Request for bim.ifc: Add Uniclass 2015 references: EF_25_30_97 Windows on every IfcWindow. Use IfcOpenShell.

First a look at what the model holds.

```python
import ifcopenshell

model = ifcopenshell.open("bim.ifc")
print(model.schema)
print("classifications:", [c.Name for c in model.by_type("IfcClassification")])
for ifc_class in ("IfcDoor", "IfcRoof", "IfcStair", "IfcWall", "IfcWindow"):
    print(ifc_class, len(model.by_type(ifc_class)))
```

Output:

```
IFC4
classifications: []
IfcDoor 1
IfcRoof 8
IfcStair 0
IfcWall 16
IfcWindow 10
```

```python
import ifcopenshell
import ifcopenshell.api.classification

model = ifcopenshell.open("bim.ifc")

system = ifcopenshell.api.classification.add_classification(model, classification="Uniclass 2015")

codes = {
    "IfcWindow": ("EF_25_30_97", "Windows"),
}
for ifc_class, (code, name) in codes.items():
    products = model.by_type(ifc_class)
    ifcopenshell.api.classification.add_reference(
        model, products=products, classification=system, identification=code, name=name
    )
    print(code, len(products))

model.write("bim_v2.ifc")
```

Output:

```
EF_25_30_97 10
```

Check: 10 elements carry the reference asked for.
